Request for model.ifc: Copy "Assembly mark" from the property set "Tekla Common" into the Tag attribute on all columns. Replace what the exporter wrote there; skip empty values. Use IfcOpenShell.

First a look at what the model holds.

```python
import ifcopenshell
import ifcopenshell.util.element

model = ifcopenshell.open("model.ifc")
print(model.schema)
columns = model.by_type("IfcColumn")
print(len(columns), "columns")
for e in columns[:8]:
    source = ifcopenshell.util.element.get_pset(e, "Tekla Common", "Assembly mark")
    target = e.Tag
    print(e.id(), repr(source), repr(target), sep=" | ")
```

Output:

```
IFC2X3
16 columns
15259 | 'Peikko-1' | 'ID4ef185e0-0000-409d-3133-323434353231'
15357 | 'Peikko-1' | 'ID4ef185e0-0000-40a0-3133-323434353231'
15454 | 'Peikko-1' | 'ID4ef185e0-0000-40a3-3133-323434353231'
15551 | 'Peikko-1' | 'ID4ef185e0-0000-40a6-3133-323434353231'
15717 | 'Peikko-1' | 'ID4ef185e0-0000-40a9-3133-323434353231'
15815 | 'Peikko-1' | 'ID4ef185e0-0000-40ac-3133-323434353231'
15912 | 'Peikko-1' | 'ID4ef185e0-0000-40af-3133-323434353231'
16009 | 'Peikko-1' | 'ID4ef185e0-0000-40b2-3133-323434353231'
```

```python
import ifcopenshell
import ifcopenshell.util.element

model = ifcopenshell.open("model.ifc")

count = 0
for e in model.by_type("IfcColumn"):
    value = ifcopenshell.util.element.get_pset(e, "Tekla Common", "Assembly mark")
    current = e.Tag
    if not value or not value.strip() or current == value:
        continue
    e.Tag = value
    count += 1

print(count, "columns updated")

model.write("model_edited.ifc")
```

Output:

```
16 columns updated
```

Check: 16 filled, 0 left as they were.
